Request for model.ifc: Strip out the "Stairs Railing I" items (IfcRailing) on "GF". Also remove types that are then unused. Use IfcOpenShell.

First a look at what the model holds.

```python
import ifcopenshell
import ifcopenshell.util.element

model = ifcopenshell.open("model.ifc")
print(model.schema)
storey = next(s for s in model.by_type("IfcBuildingStorey") if s.Name == "GF")
railings = [e for e in ifcopenshell.util.element.get_decomposition(storey) if e.is_a("IfcRailing")]
seen = {}
for e in railings:
    element_type = ifcopenshell.util.element.get_type(e)
    name = element_type.Name if element_type not in (None, e) else None
    seen[name] = seen.get(name, 0) + 1
for name, count in sorted(seen.items(), key=str):
    print(count, "x", name)
```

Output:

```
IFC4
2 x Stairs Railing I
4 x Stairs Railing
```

```python
import ifcopenshell
import ifcopenshell.api.root
import ifcopenshell.util.element

model = ifcopenshell.open("model.ifc")

storey = next(s for s in model.by_type("IfcBuildingStorey") if s.Name == "GF")
railings = [e for e in ifcopenshell.util.element.get_decomposition(storey) if e.is_a("IfcRailing")]
targets = [e for e in railings if (t := ifcopenshell.util.element.get_type(e)) not in (None, e) and t.Name == "Stairs Railing I"]
types = {ifcopenshell.util.element.get_type(e) for e in targets} - {None, *targets}

for e in targets:
    ifcopenshell.api.root.remove_product(model, product=e)
print(len(targets), "removed")

unused = [t for t in types if not ifcopenshell.util.element.get_types(t)]
for t in unused:
    ifcopenshell.api.root.remove_product(model, product=t)
print(len(unused), "unused types removed")

model.write("model-out.ifc")
```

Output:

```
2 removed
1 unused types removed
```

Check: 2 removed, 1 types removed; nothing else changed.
